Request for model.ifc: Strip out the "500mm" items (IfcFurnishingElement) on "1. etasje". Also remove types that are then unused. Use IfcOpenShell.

First a look at what the model holds.

```python
import ifcopenshell
import ifcopenshell.util.element

model = ifcopenshell.open("model.ifc")
print(model.schema)
storey = next(s for s in model.by_type("IfcBuildingStorey") if s.Name == "1. etasje")
furniture = [e for e in ifcopenshell.util.element.get_decomposition(storey) if e.is_a("IfcFurnishingElement")]
seen = {}
for e in furniture:
    element_type = ifcopenshell.util.element.get_type(e)
    name = element_type.Name if element_type not in (None, e) else None
    seen[name] = seen.get(name, 0) + 1
for name, count in sorted(seen.items(), key=str):
    print(count, "x", name)
```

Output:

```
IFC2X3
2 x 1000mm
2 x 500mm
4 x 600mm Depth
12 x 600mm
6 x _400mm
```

```python
import ifcopenshell
import ifcopenshell.api.root
import ifcopenshell.util.element

model = ifcopenshell.open("model.ifc")

storey = next(s for s in model.by_type("IfcBuildingStorey") if s.Name == "1. etasje")
furniture = [e for e in ifcopenshell.util.element.get_decomposition(storey) if e.is_a("IfcFurnishingElement")]
targets = [e for e in furniture if (t := ifcopenshell.util.element.get_type(e)) not in (None, e) and t.Name == "500mm"]
types = {ifcopenshell.util.element.get_type(e) for e in targets} - {None, *targets}

for e in targets:
    ifcopenshell.api.root.remove_product(model, product=e)
print(len(targets), "removed")

unused = [t for t in types if not ifcopenshell.util.element.get_types(t)]
for t in unused:
    ifcopenshell.api.root.remove_product(model, product=t)
print(len(unused), "unused types removed")

model.write("model_rev.ifc")
```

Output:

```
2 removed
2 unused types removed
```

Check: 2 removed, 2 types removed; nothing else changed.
